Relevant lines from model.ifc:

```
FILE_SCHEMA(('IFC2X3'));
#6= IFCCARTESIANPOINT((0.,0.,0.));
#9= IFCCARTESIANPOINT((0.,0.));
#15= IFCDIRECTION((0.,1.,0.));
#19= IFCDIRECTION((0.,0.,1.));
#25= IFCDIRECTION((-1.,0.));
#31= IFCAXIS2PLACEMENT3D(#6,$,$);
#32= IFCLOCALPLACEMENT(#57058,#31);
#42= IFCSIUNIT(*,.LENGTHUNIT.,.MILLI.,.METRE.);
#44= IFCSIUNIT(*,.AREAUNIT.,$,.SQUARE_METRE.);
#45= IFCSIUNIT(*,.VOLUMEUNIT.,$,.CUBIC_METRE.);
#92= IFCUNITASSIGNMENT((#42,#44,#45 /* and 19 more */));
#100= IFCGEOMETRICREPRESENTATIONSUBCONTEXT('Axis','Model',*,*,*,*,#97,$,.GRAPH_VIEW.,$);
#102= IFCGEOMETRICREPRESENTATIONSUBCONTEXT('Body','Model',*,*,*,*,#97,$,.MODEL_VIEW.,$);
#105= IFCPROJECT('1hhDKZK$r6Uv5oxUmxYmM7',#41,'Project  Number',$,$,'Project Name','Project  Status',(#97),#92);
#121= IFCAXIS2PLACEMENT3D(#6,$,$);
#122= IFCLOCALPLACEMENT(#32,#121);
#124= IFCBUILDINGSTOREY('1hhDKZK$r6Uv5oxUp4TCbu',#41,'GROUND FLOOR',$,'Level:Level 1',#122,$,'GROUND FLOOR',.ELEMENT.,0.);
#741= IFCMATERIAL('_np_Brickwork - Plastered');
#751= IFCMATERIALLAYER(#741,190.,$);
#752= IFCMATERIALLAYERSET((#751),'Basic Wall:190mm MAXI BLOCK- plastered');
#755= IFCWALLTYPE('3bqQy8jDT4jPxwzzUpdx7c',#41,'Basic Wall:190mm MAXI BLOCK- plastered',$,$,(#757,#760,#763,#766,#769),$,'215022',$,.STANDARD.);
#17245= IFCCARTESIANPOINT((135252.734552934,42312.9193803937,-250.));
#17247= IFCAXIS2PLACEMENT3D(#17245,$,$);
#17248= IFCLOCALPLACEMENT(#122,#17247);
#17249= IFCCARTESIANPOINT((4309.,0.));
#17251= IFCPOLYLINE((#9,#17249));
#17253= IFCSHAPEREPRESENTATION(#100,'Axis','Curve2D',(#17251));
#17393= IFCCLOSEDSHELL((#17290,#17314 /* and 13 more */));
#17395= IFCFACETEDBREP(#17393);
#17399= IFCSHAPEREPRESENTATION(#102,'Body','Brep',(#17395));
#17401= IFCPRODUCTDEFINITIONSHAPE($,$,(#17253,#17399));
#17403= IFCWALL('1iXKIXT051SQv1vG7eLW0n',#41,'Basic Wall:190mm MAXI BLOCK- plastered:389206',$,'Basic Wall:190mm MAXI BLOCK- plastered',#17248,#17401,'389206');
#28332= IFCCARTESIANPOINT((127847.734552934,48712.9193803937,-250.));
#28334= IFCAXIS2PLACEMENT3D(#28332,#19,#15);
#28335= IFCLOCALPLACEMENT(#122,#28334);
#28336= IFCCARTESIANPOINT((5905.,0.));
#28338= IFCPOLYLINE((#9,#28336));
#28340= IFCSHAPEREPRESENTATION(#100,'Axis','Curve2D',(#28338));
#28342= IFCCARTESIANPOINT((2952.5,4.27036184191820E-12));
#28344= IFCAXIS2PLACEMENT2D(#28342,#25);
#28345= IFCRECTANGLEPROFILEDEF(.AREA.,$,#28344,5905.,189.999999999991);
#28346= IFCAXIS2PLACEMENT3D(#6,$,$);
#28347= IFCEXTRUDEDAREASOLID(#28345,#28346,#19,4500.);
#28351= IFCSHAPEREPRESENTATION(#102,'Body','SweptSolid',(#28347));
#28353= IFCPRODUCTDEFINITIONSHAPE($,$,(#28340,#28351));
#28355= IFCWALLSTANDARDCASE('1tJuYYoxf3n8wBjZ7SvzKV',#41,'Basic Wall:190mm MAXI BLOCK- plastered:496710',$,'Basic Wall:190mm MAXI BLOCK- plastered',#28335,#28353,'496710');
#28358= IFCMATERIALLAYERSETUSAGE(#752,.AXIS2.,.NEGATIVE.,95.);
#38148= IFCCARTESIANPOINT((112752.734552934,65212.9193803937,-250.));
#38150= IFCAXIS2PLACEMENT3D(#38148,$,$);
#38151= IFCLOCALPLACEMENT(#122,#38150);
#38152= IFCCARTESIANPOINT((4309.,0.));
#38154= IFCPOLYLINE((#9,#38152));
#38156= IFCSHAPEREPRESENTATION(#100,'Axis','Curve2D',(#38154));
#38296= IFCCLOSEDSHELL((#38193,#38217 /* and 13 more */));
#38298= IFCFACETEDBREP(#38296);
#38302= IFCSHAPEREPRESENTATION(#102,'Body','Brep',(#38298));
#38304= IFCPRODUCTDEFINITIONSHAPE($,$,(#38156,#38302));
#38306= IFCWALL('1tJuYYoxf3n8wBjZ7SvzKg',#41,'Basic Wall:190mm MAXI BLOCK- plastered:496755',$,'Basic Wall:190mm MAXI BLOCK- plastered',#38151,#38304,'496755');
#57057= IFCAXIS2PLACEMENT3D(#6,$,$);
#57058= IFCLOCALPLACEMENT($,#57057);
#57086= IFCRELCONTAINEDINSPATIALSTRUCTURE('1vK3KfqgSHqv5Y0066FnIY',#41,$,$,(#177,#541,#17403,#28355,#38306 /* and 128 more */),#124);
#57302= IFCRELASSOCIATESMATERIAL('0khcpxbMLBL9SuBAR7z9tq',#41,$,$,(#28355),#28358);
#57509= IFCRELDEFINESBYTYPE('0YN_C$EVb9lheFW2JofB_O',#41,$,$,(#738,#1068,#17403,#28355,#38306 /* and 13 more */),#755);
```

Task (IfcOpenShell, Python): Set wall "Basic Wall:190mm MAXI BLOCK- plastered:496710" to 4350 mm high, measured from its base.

```python
import ifcopenshell
import ifcopenshell.geom
import ifcopenshell.util.representation
import ifcopenshell.util.shape
import ifcopenshell.util.unit

model = ifcopenshell.open("model.ifc")
unit_scale = ifcopenshell.util.unit.calculate_unit_scale(model)
settings = ifcopenshell.geom.settings()


def volume(element):
    """Net volume in cubic metres, openings subtracted."""
    shape = ifcopenshell.geom.create_shape(settings, element)
    return ifcopenshell.util.shape.get_volume(shape.geometry)


wall = model.by_guid("1tJuYYoxf3n8wBjZ7SvzKV")
before = volume(wall)

body = ifcopenshell.util.representation.get_representation(wall, "Model", "Body")
solid = body.Items[0]
old_height = solid.Depth
solid.Depth = 4.35 / unit_scale
after = volume(wall)

print(f"height {old_height:g} -> {solid.Depth:g}, volume {before:.3f} -> {after:.3f} m3")

model.write("model_v2.ifc")
```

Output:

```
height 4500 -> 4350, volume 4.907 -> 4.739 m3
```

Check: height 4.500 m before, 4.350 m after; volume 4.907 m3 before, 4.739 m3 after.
